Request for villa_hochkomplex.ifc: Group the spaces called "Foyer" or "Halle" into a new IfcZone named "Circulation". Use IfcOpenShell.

First a look at what the model holds.

```python
import ifcopenshell

model = ifcopenshell.open("villa_hochkomplex.ifc")
print(model.schema)
seen = {}
for space in model.by_type("IfcSpace"):
    seen[space.LongName] = seen.get(space.LongName, 0) + 1
for name, count in sorted(seen.items(), key=str):
    print(count, "x", name)
print("zones:", [z.Name for z in model.by_type("IfcZone")][:20])
```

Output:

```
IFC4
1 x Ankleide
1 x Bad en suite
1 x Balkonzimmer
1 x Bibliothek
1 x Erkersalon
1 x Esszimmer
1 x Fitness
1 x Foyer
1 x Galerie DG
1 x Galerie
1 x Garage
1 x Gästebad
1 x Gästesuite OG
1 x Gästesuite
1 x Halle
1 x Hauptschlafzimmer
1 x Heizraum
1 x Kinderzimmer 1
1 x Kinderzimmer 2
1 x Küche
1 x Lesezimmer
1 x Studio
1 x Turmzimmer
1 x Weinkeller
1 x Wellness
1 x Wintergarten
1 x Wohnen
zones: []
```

```python
import ifcopenshell
import ifcopenshell.api.group
import ifcopenshell.api.root

model = ifcopenshell.open("villa_hochkomplex.ifc")

names = {"Foyer", "Halle"}
spaces = [s for s in model.by_type("IfcSpace") if s.LongName in names]

zone = ifcopenshell.api.root.create_entity(model, ifc_class="IfcZone", name="Circulation")
ifcopenshell.api.group.assign_group(model, products=spaces, group=zone)
print(len(spaces), "spaces in", zone.Name)

model.write("villa_hochkomplex_rev.ifc")
```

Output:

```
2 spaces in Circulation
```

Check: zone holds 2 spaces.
